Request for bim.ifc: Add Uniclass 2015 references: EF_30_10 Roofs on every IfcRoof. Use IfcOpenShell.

First a look at what the model holds.

```python
import ifcopenshell

model = ifcopenshell.open("bim.ifc")
print(model.schema)
print("classifications:", [c.Name for c in model.by_type("IfcClassification")])
for ifc_class in ("IfcDoor", "IfcRoof", "IfcStair", "IfcWall", "IfcWindow"):
    print(ifc_class, len(model.by_type(ifc_class)))
```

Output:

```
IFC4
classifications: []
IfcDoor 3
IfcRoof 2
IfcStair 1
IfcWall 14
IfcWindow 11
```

```python
import ifcopenshell
import ifcopenshell.api.classification

model = ifcopenshell.open("bim.ifc")

system = ifcopenshell.api.classification.add_classification(model, classification="Uniclass 2015")

codes = {
    "IfcRoof": ("EF_30_10", "Roofs"),
}
for ifc_class, (code, name) in codes.items():
    products = model.by_type(ifc_class)
    ifcopenshell.api.classification.add_reference(
        model, products=products, classification=system, identification=code, name=name
    )
    print(code, len(products))

model.write("bim_rev.ifc")
```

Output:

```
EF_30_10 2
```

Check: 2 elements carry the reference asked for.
